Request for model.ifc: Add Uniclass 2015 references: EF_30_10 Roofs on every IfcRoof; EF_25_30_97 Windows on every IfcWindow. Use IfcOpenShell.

First a look at what the model holds.

```python
import ifcopenshell

model = ifcopenshell.open("model.ifc")
print(model.schema)
print("classifications:", [c.Name for c in model.by_type("IfcClassification")])
for ifc_class in ("IfcDoor", "IfcRoof", "IfcStair", "IfcWall", "IfcWindow"):
    print(ifc_class, len(model.by_type(ifc_class)))
```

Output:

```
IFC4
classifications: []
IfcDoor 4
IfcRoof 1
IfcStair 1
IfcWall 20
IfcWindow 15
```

```python
import ifcopenshell
import ifcopenshell.api.classification

model = ifcopenshell.open("model.ifc")

system = ifcopenshell.api.classification.add_classification(model, classification="Uniclass 2015")

codes = {
    "IfcRoof": ("EF_30_10", "Roofs"),
    "IfcWindow": ("EF_25_30_97", "Windows"),
}
for ifc_class, (code, name) in codes.items():
    products = model.by_type(ifc_class)
    ifcopenshell.api.classification.add_reference(
        model, products=products, classification=system, identification=code, name=name
    )
    print(code, len(products))

model.write("model_v2.ifc")
```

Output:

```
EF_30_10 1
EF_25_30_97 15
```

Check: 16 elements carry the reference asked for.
